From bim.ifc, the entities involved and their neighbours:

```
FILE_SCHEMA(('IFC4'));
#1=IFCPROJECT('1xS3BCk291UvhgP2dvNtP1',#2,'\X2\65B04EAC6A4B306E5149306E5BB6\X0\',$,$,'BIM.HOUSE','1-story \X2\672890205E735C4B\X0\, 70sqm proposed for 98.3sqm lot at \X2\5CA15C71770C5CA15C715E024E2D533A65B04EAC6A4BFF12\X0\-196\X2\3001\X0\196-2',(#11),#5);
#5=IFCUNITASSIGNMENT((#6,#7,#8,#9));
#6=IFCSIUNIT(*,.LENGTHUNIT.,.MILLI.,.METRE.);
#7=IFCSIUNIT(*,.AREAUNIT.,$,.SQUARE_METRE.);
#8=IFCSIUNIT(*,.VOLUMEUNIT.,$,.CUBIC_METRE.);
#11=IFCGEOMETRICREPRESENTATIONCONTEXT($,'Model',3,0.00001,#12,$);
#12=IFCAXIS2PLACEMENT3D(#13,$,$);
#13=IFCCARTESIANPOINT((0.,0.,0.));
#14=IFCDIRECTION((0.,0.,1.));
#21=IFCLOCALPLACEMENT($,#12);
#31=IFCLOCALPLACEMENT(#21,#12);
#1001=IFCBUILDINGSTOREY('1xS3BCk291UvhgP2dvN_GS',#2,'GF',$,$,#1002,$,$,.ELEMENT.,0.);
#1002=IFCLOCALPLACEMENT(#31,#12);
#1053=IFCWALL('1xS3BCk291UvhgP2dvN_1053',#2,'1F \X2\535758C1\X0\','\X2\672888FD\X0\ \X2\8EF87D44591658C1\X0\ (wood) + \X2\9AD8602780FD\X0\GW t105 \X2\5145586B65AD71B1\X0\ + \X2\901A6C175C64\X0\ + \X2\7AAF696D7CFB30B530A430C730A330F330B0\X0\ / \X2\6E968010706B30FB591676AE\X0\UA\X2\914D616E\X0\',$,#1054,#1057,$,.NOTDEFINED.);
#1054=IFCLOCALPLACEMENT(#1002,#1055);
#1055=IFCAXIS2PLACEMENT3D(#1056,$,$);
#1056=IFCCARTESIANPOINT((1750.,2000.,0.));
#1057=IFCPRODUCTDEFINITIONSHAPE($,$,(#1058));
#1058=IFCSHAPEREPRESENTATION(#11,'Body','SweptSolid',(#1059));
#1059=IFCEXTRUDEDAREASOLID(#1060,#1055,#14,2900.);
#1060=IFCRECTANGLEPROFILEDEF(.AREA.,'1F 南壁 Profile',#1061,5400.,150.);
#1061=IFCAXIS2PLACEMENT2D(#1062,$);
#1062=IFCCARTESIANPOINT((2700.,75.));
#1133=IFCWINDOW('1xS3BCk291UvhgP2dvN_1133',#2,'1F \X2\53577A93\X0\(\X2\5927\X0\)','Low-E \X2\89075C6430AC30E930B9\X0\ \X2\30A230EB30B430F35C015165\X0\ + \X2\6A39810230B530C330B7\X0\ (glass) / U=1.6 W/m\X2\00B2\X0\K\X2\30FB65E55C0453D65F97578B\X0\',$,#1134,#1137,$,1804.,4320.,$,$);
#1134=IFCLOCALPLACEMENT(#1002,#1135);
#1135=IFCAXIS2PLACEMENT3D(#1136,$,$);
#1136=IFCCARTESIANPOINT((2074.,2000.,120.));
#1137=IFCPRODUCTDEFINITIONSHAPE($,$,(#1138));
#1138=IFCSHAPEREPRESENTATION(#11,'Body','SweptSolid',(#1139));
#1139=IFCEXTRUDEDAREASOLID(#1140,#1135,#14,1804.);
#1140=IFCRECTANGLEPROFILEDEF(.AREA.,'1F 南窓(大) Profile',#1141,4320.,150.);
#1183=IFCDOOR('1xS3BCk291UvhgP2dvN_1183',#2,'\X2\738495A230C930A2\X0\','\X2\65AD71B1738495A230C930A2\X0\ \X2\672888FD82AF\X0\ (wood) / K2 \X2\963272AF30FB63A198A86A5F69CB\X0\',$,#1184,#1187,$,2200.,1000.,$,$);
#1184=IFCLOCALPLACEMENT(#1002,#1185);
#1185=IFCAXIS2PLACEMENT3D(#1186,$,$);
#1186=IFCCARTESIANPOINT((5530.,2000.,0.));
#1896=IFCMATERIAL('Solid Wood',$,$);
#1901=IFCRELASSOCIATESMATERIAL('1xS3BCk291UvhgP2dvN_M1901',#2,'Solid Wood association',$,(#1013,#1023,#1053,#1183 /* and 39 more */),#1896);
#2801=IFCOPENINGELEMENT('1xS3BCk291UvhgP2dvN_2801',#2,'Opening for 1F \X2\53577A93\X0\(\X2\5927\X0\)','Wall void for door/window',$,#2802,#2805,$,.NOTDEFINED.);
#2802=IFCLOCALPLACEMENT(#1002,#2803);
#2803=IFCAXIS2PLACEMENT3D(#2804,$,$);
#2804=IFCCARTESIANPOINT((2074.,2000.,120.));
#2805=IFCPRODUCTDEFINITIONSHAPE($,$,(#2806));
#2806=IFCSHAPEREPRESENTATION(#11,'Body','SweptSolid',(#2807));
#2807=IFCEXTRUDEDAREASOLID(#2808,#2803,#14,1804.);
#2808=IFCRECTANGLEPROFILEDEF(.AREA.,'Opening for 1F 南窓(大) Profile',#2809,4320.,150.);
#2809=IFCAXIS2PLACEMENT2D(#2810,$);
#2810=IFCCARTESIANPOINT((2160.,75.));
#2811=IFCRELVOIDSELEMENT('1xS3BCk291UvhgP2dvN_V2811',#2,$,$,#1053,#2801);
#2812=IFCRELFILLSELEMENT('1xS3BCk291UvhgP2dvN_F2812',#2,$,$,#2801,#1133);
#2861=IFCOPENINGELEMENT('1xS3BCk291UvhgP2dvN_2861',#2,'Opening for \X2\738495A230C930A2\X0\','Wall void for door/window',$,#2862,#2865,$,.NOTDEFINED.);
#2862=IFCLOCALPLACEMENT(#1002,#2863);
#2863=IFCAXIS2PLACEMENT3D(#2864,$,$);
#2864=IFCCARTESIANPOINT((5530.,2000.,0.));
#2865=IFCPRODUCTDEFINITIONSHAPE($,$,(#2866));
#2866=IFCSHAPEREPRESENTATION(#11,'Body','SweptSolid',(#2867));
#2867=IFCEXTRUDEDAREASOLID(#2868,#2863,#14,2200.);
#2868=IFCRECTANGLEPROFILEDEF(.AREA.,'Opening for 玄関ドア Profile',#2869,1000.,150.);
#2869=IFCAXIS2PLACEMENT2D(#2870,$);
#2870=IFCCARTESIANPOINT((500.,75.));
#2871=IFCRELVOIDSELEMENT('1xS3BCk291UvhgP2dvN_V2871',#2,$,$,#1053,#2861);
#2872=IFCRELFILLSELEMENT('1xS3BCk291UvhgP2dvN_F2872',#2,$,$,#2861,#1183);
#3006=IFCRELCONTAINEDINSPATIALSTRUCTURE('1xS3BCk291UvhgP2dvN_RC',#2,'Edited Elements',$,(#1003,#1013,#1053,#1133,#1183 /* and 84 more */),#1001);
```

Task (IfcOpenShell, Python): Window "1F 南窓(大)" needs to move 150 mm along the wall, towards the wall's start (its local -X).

```python
import ifcopenshell
import ifcopenshell.api.geometry
import ifcopenshell.util.placement

model = ifcopenshell.open("bim.ifc")

window = model.by_guid("1xS3BCk291UvhgP2dvN_1133")
opening = window.FillsVoids[0].RelatingOpeningElement
wall = opening.VoidsElements[0].RelatingBuildingElement

wall_matrix = ifcopenshell.util.placement.get_local_placement(wall.ObjectPlacement)
shift = wall_matrix[:3, 0] * -150.0
before = ifcopenshell.util.placement.get_local_placement(window.ObjectPlacement)[:3, 3].copy()

# The window is not placed relative to its opening, so move both.
for product in (opening, window):
    matrix = ifcopenshell.util.placement.get_local_placement(product.ObjectPlacement)
    matrix[:3, 3] += shift
    ifcopenshell.api.geometry.edit_object_placement(model, product=product, matrix=matrix, is_si=False)

after = ifcopenshell.util.placement.get_local_placement(window.ObjectPlacement)[:3, 3]
print("window moved by", (after - before).round(3) + 0.0)

model.write("bim_edited.ifc")
```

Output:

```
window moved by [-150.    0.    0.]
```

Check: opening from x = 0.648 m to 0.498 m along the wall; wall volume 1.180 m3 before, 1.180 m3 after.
